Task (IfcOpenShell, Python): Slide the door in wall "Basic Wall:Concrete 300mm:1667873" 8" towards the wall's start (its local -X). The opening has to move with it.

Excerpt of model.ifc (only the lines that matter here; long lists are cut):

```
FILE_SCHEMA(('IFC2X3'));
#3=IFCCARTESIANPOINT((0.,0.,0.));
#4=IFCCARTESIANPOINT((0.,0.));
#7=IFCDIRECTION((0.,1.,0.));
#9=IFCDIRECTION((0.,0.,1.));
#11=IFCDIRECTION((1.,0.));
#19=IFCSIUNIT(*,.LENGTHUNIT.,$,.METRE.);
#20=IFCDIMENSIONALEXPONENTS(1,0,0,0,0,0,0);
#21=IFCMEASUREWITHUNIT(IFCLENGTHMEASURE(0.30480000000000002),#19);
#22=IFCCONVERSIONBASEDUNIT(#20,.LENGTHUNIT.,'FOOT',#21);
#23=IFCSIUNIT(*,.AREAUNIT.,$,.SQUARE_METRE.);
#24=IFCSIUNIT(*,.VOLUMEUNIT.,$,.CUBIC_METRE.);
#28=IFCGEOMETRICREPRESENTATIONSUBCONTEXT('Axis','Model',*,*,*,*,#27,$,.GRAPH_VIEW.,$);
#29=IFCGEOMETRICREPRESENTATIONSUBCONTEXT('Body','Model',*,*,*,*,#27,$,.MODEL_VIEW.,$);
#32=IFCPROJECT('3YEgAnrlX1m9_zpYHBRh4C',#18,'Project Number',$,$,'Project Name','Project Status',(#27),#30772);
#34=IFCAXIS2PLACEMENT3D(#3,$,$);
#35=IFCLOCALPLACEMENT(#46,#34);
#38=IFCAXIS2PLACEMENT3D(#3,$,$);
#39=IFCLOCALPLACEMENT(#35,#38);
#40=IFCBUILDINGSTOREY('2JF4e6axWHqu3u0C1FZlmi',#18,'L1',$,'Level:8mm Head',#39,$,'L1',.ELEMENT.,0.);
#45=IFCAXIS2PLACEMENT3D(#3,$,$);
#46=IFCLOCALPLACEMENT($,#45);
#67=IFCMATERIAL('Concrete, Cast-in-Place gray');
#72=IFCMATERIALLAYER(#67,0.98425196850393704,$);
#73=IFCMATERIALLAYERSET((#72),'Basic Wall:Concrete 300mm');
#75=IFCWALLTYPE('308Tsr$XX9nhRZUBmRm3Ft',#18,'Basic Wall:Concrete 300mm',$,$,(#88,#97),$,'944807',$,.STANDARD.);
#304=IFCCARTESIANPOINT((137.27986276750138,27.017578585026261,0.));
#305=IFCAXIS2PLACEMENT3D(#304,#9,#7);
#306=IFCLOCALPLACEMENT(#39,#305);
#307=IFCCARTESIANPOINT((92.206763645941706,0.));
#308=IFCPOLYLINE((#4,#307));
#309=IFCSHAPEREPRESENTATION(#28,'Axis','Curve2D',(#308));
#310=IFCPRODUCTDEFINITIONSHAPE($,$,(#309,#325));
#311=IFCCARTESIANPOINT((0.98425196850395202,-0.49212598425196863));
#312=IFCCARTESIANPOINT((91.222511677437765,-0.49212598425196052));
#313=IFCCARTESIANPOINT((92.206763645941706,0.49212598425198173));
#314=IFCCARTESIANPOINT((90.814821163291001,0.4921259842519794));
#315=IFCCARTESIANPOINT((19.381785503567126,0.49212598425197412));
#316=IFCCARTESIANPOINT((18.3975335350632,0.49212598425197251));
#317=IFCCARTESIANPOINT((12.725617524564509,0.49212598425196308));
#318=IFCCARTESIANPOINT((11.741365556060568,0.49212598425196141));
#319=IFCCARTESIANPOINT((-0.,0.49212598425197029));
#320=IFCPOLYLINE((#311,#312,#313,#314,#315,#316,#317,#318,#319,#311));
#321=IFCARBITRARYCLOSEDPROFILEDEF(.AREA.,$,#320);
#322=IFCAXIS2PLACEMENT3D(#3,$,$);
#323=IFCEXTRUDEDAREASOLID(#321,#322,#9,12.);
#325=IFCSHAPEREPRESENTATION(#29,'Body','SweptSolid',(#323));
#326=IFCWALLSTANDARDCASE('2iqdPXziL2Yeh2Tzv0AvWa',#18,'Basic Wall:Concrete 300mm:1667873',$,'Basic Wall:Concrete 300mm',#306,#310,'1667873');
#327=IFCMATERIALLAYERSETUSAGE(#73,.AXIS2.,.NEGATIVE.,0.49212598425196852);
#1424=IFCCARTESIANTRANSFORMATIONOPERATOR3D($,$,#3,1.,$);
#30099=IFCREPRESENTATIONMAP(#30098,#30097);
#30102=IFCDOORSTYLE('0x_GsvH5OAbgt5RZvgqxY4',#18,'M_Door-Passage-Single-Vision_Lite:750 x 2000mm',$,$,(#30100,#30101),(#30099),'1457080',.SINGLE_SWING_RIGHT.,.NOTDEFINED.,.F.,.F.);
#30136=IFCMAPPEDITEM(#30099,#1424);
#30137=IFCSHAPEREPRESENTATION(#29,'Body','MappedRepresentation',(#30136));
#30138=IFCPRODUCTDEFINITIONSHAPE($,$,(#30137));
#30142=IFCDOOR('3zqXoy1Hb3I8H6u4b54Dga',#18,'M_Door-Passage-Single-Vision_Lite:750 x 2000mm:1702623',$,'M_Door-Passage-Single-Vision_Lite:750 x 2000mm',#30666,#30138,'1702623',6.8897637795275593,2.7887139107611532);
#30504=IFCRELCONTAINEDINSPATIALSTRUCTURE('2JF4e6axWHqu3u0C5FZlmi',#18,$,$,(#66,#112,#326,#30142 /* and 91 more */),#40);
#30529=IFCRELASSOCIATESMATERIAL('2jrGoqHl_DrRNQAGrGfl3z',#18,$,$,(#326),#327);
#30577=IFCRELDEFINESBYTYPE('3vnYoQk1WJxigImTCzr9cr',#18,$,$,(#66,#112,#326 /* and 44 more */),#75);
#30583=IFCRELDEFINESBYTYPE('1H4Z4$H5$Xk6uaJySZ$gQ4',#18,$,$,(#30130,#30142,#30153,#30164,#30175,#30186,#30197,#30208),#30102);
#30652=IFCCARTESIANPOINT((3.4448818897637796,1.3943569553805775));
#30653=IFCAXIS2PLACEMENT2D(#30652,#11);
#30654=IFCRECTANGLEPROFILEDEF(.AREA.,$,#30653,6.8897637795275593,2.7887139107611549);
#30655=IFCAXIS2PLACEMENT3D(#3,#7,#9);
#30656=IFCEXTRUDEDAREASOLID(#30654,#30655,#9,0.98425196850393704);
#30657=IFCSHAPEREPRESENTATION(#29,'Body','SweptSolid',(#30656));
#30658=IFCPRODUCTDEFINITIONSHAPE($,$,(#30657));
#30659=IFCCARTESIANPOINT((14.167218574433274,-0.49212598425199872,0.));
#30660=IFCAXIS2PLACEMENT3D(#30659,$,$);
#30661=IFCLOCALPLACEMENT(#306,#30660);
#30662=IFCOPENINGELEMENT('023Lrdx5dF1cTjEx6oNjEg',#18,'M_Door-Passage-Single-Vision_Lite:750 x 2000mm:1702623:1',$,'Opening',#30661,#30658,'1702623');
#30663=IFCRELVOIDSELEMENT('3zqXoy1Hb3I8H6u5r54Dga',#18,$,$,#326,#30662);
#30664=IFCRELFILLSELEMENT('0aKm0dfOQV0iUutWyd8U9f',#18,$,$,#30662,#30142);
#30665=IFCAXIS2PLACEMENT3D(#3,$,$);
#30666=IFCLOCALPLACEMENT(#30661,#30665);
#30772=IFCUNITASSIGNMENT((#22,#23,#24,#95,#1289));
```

```python
import ifcopenshell
import ifcopenshell.api.geometry
import ifcopenshell.util.placement
import ifcopenshell.util.unit

model = ifcopenshell.open("model.ifc")
unit_scale = ifcopenshell.util.unit.calculate_unit_scale(model)

door = model.by_guid("3zqXoy1Hb3I8H6u4b54Dga")
opening = door.FillsVoids[0].RelatingOpeningElement
wall = opening.VoidsElements[0].RelatingBuildingElement

wall_matrix = ifcopenshell.util.placement.get_local_placement(wall.ObjectPlacement)
shift = wall_matrix[:3, 0] * -8 * 0.0254 / unit_scale
before = ifcopenshell.util.placement.get_local_placement(door.ObjectPlacement)[:3, 3].copy()

# The door is placed relative to its opening, so it follows when the opening moves.
matrix = ifcopenshell.util.placement.get_local_placement(opening.ObjectPlacement)
matrix[:3, 3] += shift
ifcopenshell.api.geometry.edit_object_placement(
    model, product=opening, matrix=matrix, is_si=False, should_transform_children=True
)

after = ifcopenshell.util.placement.get_local_placement(door.ObjectPlacement)[:3, 3]
print("door moved by", (after - before).round(3) + 0.0)

model.write("model_edited.ifc")
```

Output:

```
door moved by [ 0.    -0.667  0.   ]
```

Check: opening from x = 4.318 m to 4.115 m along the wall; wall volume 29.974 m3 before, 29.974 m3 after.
